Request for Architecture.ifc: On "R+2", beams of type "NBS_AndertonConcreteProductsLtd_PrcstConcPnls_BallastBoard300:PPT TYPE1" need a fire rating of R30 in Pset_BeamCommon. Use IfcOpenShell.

First a look at what the model holds.

```python
import ifcopenshell
import ifcopenshell.util.element

model = ifcopenshell.open("Architecture.ifc")
print(model.schema)
storey = next(s for s in model.by_type("IfcBuildingStorey") if s.Name == "R+2")
beams = [e for e in ifcopenshell.util.element.get_decomposition(storey) if e.is_a("IfcBeam")]
seen = {}
for e in beams:
    element_type = ifcopenshell.util.element.get_type(e)
    key = (element_type.Name if element_type != e and element_type else None, ifcopenshell.util.element.get_pset(e, "Pset_BeamCommon", "FireRating"))
    seen[key] = seen.get(key, 0) + 1
for (name, value), count in sorted(seen.items(), key=str):
    print(count, "x", name, "|", value)
```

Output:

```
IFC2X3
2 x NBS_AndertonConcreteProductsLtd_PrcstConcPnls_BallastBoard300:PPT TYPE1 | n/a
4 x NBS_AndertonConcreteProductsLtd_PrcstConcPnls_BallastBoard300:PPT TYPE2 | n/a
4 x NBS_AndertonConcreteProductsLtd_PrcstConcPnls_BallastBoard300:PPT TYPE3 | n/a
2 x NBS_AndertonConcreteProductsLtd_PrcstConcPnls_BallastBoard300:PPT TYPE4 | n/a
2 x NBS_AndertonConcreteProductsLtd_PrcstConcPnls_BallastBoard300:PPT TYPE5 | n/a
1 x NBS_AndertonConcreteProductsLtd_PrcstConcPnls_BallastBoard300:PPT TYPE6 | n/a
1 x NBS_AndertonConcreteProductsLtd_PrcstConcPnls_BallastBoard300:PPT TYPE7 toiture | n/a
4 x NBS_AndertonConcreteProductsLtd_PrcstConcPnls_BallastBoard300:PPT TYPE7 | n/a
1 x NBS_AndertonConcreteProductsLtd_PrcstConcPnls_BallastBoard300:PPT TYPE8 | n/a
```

```python
import ifcopenshell
import ifcopenshell.api.pset
import ifcopenshell.util.element

model = ifcopenshell.open("Architecture.ifc")

storey = next(s for s in model.by_type("IfcBuildingStorey") if s.Name == "R+2")
beams = [e for e in ifcopenshell.util.element.get_decomposition(storey) if e.is_a("IfcBeam")]

count = 0
for e in beams:
    element_type = ifcopenshell.util.element.get_type(e)
    if element_type in (None, e) or element_type.Name != "NBS_AndertonConcreteProductsLtd_PrcstConcPnls_BallastBoard300:PPT TYPE1":
        continue
    # add_pset returns the element's existing set when there is one.
    pset = ifcopenshell.api.pset.add_pset(model, product=e, name="Pset_BeamCommon")
    ifcopenshell.api.pset.edit_pset(model, pset=pset, properties={"FireRating": "R30"})
    count += 1

print(count, "beams updated")

model.write("Architecture_updated.ifc")
```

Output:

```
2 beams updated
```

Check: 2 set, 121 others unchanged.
